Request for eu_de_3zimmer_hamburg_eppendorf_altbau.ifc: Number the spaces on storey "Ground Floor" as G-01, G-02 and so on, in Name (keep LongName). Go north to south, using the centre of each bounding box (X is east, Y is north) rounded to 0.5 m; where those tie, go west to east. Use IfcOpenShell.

First a look at what the model holds.

```python
import ifcopenshell
import ifcopenshell.util.element
import ifcopenshell.util.placement

model = ifcopenshell.open("eu_de_3zimmer_hamburg_eppendorf_altbau.ifc")
print(model.schema)
storey = next(s for s in model.by_type("IfcBuildingStorey") if s.Name == "Ground Floor")
spaces = [e for e in ifcopenshell.util.element.get_decomposition(storey) if e.is_a("IfcSpace")]
for e in sorted(spaces, key=lambda e: e.id()):
    origin = ifcopenshell.util.placement.get_local_placement(e.ObjectPlacement)[:3, 3]
    print(e.id(), e.Name, e.LongName, origin.round(2) + 0.0, sep=" | ")
```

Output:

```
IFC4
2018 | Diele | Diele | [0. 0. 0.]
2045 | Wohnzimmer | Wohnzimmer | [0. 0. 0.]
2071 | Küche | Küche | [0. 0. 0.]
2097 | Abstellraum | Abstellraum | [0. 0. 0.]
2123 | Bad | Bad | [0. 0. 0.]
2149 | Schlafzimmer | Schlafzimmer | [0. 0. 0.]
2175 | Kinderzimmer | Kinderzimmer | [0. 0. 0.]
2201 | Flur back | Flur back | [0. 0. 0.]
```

```python
import ifcopenshell
import ifcopenshell.geom
import ifcopenshell.util.element
import ifcopenshell.util.shape

model = ifcopenshell.open("eu_de_3zimmer_hamburg_eppendorf_altbau.ifc")
settings = ifcopenshell.geom.settings()
settings.set("use-world-coords", True)


def centre(element):
    shape = ifcopenshell.geom.create_shape(settings, element)
    return ifcopenshell.util.shape.get_bbox_centroid(shape.geometry)


storey = next(s for s in model.by_type("IfcBuildingStorey") if s.Name == "Ground Floor")
spaces = [e for e in ifcopenshell.util.element.get_decomposition(storey) if e.is_a("IfcSpace")]

# Insertion points can sit at a corner or the storey origin, so sort by the geometry (in metres).
centres = {e: centre(e) for e in spaces}
spaces.sort(key=lambda e: (-round(centres[e][1] / 0.5), centres[e][0]))

for i, e in enumerate(spaces, start=1):
    number = f"G-{i:02d}"
    e.Name = number
    print(e.id(), number)

model.write("eu_de_3zimmer_hamburg_eppendorf_altbau_rev.ifc")
```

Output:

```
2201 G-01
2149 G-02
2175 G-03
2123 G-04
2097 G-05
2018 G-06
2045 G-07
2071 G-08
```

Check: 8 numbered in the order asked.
